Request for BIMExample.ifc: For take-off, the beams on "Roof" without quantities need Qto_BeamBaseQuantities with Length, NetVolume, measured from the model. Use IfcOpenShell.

First a look at what the model holds.

```python
import ifcopenshell
import ifcopenshell.util.element
import ifcopenshell.util.unit

model = ifcopenshell.open("BIMExample.ifc")
print(model.schema)
for unit_type in ("LENGTHUNIT", "AREAUNIT", "VOLUMEUNIT"):
    print(unit_type, ifcopenshell.util.unit.calculate_unit_scale(model, unit_type))
storey = next(s for s in model.by_type("IfcBuildingStorey") if s.Name == "Roof")
beams = [e for e in ifcopenshell.util.element.get_decomposition(storey) if e.is_a("IfcBeam")]
for e in sorted(beams, key=lambda e: e.id()):
    print(e.id(), e.is_a(), e.Name, list(ifcopenshell.util.element.get_psets(e, qtos_only=True)), sep=" | ")
```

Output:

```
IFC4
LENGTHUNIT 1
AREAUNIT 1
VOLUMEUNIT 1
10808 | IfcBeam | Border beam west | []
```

```python
import ifcopenshell
import ifcopenshell.api.pset
import ifcopenshell.geom
import ifcopenshell.util.element
import ifcopenshell.util.shape
import ifcopenshell.util.unit

model = ifcopenshell.open("BIMExample.ifc")
unit_scale = ifcopenshell.util.unit.calculate_unit_scale(model)
volume_scale = ifcopenshell.util.unit.calculate_unit_scale(model, "VOLUMEUNIT")
settings = ifcopenshell.geom.settings()

storey = next(s for s in model.by_type("IfcBuildingStorey") if s.Name == "Roof")
beams = [e for e in ifcopenshell.util.element.get_decomposition(storey) if e.is_a("IfcBeam")]

for e in sorted(beams, key=lambda e: e.id()):
    if ifcopenshell.util.element.get_psets(e, qtos_only=True, should_inherit=False):
        continue
    # Geometry comes back in metres, in the element's own axes.
    shape = ifcopenshell.geom.create_shape(settings, e)
    values = {
        "Length": ifcopenshell.util.shape.get_max_xyz(shape.geometry) / unit_scale,
        "NetVolume": ifcopenshell.util.shape.get_volume(shape.geometry) / volume_scale,
    }
    qto = ifcopenshell.api.pset.add_qto(model, product=e, name="Qto_BeamBaseQuantities")
    ifcopenshell.api.pset.edit_qto(model, qto=qto, properties=values)
    print(e.id(), {k: round(v, 3) for k, v in values.items()})

model.write("BIMExample_edited.ifc")
```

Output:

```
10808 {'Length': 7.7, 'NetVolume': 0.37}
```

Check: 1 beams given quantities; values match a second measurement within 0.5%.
